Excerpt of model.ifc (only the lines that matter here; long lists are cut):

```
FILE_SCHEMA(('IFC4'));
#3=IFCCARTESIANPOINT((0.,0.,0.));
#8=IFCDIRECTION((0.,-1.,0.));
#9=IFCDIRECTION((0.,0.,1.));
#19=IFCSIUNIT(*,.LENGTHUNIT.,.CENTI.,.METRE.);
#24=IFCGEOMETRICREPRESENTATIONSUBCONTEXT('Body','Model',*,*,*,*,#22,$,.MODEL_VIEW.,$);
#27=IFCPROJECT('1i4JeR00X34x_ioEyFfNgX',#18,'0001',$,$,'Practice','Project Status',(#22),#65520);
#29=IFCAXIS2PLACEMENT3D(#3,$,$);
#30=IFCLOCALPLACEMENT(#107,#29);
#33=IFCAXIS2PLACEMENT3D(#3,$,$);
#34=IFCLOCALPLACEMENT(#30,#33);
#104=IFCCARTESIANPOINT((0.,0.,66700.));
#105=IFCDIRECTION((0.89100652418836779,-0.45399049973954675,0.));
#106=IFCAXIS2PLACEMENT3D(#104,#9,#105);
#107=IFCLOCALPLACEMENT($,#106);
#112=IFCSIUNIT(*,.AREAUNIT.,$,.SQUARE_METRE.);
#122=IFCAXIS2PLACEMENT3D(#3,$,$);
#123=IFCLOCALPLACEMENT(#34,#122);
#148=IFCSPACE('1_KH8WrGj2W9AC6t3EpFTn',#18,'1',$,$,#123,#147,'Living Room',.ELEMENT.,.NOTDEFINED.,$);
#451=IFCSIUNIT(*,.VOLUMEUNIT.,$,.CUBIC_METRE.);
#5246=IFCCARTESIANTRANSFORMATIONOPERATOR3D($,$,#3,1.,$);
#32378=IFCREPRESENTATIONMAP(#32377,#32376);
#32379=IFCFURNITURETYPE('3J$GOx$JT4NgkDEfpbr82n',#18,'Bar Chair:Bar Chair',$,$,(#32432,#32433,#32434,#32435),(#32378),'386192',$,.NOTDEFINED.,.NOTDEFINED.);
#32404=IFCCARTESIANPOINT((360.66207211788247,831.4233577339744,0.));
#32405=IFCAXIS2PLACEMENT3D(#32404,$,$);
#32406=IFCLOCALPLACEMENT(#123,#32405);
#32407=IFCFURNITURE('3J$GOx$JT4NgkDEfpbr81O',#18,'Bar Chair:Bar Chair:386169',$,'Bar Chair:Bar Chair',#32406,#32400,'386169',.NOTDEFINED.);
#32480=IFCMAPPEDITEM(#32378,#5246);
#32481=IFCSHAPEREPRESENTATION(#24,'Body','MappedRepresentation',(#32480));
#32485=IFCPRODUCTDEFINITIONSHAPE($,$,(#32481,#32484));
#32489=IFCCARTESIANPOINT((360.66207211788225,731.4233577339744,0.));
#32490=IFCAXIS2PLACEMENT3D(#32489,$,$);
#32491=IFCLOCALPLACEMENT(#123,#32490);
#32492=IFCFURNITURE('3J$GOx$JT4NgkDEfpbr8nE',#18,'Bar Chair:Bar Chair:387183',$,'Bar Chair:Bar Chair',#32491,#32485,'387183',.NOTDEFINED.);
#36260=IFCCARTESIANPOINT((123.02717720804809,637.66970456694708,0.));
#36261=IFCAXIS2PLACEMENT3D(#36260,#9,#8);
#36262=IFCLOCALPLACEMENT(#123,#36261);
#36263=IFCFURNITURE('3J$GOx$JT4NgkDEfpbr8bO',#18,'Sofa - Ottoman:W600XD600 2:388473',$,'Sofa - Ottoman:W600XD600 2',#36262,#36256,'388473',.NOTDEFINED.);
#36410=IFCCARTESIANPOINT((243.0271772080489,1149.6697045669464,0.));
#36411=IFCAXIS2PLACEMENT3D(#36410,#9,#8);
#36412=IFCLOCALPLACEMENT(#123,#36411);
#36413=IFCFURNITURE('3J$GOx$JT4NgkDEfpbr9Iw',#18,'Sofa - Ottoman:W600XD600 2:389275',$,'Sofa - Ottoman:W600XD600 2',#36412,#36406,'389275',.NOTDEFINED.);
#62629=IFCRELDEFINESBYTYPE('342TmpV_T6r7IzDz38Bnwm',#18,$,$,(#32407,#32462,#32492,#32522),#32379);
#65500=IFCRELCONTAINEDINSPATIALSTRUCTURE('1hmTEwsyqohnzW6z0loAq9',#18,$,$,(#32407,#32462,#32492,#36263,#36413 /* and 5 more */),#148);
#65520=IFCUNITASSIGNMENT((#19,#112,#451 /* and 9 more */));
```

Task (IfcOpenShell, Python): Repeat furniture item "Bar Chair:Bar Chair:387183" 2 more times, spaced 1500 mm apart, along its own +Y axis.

```python
import ifcopenshell
import ifcopenshell.api.geometry
import ifcopenshell.api.root
import ifcopenshell.util.element
import ifcopenshell.util.placement
import ifcopenshell.util.unit

model = ifcopenshell.open("model.ifc")
unit_scale = ifcopenshell.util.unit.calculate_unit_scale(model)


def reuse_history(source, copy):
    """copy_class also copies each property set's owner history, people and application; keep the originals."""
    for rel in copy.IsDefinedBy:
        if rel.is_a("IfcRelDefinesByProperties") and (history := rel.RelatingPropertyDefinition.OwnerHistory):
            rel.RelatingPropertyDefinition.OwnerHistory = source.OwnerHistory
            ifcopenshell.util.element.remove_deep2(model, history)


source = model.by_id(32492)
base = ifcopenshell.util.placement.get_local_placement(source.ObjectPlacement)
step = base[:3, 1] * 1.5 / unit_scale

for i in range(1, 3):
    copy = ifcopenshell.api.root.copy_class(model, product=source)
    copy.Representation = ifcopenshell.util.element.copy_deep(
        model, source.Representation, exclude=["IfcGeometricRepresentationContext", "IfcRepresentationMap"]
    )
    copy.Name = "Bar Chair:Bar Chair"
    copy.Tag = None
    reuse_history(source, copy)
    matrix = base.copy()
    matrix[:3, 3] += i * step
    print("added at", matrix[:3, 3].round(3) + 0.0)
    ifcopenshell.api.geometry.edit_object_placement(model, product=copy, matrix=matrix, is_si=False)

model.write("model_edited.ifc")
```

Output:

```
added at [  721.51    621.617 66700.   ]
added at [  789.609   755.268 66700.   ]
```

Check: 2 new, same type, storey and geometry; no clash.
